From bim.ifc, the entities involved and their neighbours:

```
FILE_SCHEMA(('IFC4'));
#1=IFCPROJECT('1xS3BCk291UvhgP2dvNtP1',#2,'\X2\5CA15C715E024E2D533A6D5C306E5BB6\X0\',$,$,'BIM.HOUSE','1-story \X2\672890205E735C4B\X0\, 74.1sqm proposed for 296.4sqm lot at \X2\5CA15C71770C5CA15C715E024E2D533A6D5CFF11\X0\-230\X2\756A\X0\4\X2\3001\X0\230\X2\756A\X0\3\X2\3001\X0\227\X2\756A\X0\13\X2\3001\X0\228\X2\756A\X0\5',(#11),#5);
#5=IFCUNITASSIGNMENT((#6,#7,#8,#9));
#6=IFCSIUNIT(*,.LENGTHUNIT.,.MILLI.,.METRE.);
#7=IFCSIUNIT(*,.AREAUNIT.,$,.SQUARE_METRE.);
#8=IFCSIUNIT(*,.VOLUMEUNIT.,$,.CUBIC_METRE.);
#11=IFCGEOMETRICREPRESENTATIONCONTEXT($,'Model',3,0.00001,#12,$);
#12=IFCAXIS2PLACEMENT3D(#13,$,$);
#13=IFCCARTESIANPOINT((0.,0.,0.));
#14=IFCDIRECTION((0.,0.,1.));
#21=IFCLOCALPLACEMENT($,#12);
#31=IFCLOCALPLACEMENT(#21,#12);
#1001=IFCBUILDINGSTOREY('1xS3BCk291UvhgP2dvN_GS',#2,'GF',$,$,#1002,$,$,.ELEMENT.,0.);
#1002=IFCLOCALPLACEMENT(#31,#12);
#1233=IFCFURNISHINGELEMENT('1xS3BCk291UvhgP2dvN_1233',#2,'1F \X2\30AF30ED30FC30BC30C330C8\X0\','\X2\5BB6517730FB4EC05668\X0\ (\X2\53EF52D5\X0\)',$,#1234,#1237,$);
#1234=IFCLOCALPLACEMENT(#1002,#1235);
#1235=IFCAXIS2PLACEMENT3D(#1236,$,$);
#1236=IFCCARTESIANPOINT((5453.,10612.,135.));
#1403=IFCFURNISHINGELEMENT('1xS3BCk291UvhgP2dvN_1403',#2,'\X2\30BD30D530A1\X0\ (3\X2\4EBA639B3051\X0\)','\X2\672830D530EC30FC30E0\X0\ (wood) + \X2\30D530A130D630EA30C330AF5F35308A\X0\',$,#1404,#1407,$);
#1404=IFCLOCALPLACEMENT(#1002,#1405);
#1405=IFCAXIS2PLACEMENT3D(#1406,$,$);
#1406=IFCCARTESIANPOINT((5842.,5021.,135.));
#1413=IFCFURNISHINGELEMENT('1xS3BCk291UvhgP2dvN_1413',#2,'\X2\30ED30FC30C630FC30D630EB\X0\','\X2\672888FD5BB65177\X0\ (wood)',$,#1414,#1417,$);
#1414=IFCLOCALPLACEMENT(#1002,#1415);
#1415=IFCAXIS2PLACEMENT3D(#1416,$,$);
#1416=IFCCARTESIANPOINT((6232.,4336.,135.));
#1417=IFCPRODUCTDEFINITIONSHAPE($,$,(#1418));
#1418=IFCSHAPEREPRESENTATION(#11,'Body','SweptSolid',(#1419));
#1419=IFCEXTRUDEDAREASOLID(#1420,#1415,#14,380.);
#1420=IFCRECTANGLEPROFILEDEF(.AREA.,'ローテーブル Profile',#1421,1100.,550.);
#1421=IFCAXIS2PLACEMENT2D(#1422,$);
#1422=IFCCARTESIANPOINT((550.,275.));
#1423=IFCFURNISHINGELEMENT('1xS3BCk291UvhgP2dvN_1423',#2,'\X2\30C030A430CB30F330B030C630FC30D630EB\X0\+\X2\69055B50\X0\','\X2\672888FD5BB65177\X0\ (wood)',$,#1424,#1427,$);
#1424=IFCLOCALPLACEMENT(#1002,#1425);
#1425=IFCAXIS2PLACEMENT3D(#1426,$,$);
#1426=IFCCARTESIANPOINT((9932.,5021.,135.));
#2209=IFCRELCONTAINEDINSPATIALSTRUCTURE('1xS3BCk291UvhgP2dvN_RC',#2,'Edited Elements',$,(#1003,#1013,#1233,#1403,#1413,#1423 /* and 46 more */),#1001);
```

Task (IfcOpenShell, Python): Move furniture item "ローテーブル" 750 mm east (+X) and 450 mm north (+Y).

```python
import ifcopenshell
import ifcopenshell.api.geometry
import ifcopenshell.util.placement

model = ifcopenshell.open("bim.ifc")

item = model.by_guid("1xS3BCk291UvhgP2dvN_1413")
matrix = ifcopenshell.util.placement.get_local_placement(item.ObjectPlacement)
matrix[0, 3] += 750.0
matrix[1, 3] += 450.0
ifcopenshell.api.geometry.edit_object_placement(model, product=item, matrix=matrix, is_si=False)

print(ifcopenshell.util.placement.get_local_placement(item.ObjectPlacement).round(3) + 0.0)

model.write("bim_rev.ifc")
```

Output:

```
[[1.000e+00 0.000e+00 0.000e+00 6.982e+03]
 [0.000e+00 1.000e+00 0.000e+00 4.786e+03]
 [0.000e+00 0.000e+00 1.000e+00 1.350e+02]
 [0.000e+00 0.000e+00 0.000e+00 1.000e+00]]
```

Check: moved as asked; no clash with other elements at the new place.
